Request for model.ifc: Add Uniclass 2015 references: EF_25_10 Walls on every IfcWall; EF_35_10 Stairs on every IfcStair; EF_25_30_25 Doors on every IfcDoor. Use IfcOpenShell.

First a look at what the model holds.

```python
import ifcopenshell

model = ifcopenshell.open("model.ifc")
print(model.schema)
print("classifications:", [c.Name for c in model.by_type("IfcClassification")])
for ifc_class in ("IfcDoor", "IfcRoof", "IfcStair", "IfcWall", "IfcWindow"):
    print(ifc_class, len(model.by_type(ifc_class)))
```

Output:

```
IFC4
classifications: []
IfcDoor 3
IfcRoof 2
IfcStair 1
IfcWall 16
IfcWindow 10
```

```python
import ifcopenshell
import ifcopenshell.api.classification

model = ifcopenshell.open("model.ifc")

system = ifcopenshell.api.classification.add_classification(model, classification="Uniclass 2015")

codes = {
    "IfcWall": ("EF_25_10", "Walls"),
    "IfcStair": ("EF_35_10", "Stairs"),
    "IfcDoor": ("EF_25_30_25", "Doors"),
}
for ifc_class, (code, name) in codes.items():
    products = model.by_type(ifc_class)
    ifcopenshell.api.classification.add_reference(
        model, products=products, classification=system, identification=code, name=name
    )
    print(code, len(products))

model.write("model_updated.ifc")
```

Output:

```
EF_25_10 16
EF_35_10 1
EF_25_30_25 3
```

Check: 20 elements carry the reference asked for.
